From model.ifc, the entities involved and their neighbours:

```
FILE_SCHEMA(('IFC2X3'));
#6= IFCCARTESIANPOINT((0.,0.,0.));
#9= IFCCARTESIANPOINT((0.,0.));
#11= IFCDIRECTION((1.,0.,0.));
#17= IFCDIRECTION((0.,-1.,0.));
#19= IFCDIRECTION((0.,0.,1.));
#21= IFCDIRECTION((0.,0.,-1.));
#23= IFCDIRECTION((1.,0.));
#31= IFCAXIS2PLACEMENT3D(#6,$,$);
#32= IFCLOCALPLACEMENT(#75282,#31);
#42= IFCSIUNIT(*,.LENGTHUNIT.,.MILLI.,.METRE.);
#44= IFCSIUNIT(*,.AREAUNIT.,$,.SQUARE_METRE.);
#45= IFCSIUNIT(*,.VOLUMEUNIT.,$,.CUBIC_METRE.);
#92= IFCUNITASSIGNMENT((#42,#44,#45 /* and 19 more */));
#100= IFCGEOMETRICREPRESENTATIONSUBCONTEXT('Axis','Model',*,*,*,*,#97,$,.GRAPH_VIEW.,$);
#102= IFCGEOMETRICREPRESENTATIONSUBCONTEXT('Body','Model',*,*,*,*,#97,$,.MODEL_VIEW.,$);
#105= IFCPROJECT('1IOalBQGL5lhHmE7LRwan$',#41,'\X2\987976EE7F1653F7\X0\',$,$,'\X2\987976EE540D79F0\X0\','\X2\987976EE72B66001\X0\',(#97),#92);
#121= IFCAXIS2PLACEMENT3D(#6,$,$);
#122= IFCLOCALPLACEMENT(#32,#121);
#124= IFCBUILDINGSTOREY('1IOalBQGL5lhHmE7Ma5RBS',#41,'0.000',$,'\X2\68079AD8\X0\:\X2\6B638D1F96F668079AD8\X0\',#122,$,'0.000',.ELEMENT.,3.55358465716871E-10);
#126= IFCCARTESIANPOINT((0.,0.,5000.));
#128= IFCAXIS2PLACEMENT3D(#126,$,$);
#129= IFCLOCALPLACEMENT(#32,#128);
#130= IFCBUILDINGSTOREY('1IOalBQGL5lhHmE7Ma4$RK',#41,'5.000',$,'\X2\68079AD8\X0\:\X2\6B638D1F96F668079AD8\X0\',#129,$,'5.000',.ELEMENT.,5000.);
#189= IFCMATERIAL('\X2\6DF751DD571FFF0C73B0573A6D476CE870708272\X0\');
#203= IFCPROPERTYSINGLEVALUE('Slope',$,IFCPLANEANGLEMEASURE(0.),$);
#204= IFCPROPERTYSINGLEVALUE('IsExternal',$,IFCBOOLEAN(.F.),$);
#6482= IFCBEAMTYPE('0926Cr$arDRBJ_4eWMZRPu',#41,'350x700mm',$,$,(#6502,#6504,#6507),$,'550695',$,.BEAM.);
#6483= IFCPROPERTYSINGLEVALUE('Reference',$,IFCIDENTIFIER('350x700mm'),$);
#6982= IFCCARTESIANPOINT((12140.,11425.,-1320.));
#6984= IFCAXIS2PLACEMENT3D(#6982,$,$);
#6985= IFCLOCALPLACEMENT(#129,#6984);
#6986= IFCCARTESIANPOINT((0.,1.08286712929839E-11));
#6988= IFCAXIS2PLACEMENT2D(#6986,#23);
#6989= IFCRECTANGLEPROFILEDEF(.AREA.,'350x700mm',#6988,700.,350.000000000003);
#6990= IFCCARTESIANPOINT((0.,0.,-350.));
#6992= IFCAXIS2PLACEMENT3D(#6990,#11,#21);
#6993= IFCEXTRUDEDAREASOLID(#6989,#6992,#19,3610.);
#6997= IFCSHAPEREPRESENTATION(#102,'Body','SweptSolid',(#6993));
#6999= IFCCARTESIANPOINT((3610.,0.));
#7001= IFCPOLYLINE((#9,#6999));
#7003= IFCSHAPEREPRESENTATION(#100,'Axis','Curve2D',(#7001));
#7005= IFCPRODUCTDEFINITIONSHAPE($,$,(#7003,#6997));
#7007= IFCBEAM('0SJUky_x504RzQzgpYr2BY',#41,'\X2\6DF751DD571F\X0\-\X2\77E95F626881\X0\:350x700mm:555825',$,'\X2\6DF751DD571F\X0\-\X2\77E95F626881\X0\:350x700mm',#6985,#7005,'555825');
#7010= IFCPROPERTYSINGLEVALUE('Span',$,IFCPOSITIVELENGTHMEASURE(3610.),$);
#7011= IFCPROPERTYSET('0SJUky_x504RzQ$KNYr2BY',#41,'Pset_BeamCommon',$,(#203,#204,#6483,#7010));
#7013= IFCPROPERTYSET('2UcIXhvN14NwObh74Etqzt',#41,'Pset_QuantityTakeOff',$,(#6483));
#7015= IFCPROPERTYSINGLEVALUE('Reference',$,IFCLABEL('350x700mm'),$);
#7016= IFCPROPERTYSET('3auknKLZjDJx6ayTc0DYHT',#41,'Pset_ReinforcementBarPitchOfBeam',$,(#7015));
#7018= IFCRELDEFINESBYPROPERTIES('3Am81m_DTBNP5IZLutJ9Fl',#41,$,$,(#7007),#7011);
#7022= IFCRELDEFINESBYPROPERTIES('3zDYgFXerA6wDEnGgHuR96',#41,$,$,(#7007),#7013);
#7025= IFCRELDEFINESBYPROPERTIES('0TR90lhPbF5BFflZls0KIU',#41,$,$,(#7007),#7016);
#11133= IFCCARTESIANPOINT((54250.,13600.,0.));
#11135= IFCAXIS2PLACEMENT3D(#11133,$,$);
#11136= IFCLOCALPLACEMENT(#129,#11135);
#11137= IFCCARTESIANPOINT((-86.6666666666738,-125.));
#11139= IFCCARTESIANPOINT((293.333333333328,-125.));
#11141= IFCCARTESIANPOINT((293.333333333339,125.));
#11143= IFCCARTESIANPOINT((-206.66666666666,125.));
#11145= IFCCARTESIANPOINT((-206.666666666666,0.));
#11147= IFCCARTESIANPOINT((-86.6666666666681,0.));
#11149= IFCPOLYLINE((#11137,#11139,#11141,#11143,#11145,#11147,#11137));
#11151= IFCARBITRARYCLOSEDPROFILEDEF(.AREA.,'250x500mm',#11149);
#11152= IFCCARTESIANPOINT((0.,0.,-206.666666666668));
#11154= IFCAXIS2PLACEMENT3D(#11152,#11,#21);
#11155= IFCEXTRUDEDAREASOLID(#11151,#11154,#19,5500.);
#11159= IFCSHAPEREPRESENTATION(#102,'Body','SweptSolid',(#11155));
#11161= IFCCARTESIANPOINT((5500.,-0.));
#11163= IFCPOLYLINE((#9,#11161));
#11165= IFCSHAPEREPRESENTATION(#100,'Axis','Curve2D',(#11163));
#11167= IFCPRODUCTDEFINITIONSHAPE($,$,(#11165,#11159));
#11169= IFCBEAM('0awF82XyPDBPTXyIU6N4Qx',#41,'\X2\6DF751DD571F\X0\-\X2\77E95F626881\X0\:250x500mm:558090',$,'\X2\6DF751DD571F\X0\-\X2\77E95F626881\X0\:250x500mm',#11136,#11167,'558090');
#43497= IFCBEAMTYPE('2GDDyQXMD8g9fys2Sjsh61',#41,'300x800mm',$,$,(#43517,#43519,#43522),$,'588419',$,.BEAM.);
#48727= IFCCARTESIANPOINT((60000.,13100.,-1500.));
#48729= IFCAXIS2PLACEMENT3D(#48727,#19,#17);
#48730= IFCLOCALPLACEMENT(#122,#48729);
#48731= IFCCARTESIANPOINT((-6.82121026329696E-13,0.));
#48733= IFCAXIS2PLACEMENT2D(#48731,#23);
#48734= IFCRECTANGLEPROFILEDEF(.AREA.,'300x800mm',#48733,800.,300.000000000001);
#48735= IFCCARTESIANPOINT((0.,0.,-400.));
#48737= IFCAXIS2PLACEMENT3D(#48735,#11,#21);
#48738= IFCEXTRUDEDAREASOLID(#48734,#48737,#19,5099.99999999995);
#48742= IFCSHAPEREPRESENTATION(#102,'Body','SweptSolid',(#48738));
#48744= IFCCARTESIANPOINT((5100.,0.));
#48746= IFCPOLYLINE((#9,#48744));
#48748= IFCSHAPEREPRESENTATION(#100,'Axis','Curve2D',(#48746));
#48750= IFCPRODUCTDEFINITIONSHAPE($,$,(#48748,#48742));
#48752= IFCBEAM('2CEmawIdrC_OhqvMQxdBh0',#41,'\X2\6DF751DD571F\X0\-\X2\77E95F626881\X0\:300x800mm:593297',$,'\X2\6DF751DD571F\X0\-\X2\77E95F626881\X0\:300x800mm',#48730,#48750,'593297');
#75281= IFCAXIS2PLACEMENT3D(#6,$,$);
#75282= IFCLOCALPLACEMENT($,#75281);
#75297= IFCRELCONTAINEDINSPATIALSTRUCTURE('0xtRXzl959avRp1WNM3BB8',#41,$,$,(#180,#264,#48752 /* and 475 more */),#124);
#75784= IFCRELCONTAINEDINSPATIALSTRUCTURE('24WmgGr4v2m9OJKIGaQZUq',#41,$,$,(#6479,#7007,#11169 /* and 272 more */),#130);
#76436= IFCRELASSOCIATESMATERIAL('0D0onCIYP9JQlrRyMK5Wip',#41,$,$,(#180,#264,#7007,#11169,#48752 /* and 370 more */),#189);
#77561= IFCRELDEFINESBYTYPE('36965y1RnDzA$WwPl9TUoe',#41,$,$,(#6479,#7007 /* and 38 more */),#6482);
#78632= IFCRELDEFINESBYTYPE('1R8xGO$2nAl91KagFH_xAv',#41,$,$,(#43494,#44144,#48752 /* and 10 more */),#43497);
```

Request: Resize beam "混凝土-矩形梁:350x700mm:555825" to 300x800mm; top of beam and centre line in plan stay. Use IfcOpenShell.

```python
import ifcopenshell
import ifcopenshell.api.pset
import ifcopenshell.api.type
import ifcopenshell.util.element
import ifcopenshell.util.representation

model = ifcopenshell.open("model.ifc")

member = model.by_guid("0SJUky_x504RzQzgpYr2BY")
source = next(p for p in model.by_type("IfcRectangleProfileDef") if p.ProfileName == "300x800mm")

body = ifcopenshell.util.representation.get_representation(member, "Model", "Body")
solid = body.Items[0]
old_profile = solid.SweptArea

# Copy the section's sizes but keep this member's own profile position.
profile = ifcopenshell.util.element.copy(model, source)
# Profiles are centred, so shift by half the change in depth to hold the top.
shift = (old_profile.XDim - profile.XDim) / 2
x, y = old_profile.Position.Location.Coordinates
up = (-1.0, 0.0)  # upwards, in the solid's own plane
location = model.createIfcCartesianPoint((x + up[0] * shift, y + up[1] * shift))
profile.Position = model.createIfcAxis2Placement2D(location, old_profile.Position.RefDirection)
solid.SweptArea = profile
if not model.get_total_inverses(old_profile):
    ifcopenshell.util.element.remove_deep2(model, old_profile)

new_type = model.by_guid("2GDDyQXMD8g9fys2Sjsh61")
ifcopenshell.api.type.assign_type(
    model, related_objects=[member], relating_type=new_type, should_map_representations=False
)
member.Name = member.Name.replace("350x700mm", "300x800mm")
member.ObjectType = "混凝土-矩形梁:300x800mm"
pset = model.by_id(ifcopenshell.util.element.get_pset(member, "Pset_BeamCommon", should_inherit=False)["id"])
ifcopenshell.api.pset.edit_pset(model, pset=pset, properties={"Reference": "300x800mm"})
pset = model.by_id(ifcopenshell.util.element.get_pset(member, "Pset_QuantityTakeOff", should_inherit=False)["id"])
ifcopenshell.api.pset.edit_pset(model, pset=pset, properties={"Reference": "300x800mm"})
pset = model.by_id(ifcopenshell.util.element.get_pset(member, "Pset_ReinforcementBarPitchOfBeam", should_inherit=False)["id"])
ifcopenshell.api.pset.edit_pset(model, pset=pset, properties={"Reference": "300x800mm"})

print(solid.SweptArea)

model.write("model_updated.ifc")
```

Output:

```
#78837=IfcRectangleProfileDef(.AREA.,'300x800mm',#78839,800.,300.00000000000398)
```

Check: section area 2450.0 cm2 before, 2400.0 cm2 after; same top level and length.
